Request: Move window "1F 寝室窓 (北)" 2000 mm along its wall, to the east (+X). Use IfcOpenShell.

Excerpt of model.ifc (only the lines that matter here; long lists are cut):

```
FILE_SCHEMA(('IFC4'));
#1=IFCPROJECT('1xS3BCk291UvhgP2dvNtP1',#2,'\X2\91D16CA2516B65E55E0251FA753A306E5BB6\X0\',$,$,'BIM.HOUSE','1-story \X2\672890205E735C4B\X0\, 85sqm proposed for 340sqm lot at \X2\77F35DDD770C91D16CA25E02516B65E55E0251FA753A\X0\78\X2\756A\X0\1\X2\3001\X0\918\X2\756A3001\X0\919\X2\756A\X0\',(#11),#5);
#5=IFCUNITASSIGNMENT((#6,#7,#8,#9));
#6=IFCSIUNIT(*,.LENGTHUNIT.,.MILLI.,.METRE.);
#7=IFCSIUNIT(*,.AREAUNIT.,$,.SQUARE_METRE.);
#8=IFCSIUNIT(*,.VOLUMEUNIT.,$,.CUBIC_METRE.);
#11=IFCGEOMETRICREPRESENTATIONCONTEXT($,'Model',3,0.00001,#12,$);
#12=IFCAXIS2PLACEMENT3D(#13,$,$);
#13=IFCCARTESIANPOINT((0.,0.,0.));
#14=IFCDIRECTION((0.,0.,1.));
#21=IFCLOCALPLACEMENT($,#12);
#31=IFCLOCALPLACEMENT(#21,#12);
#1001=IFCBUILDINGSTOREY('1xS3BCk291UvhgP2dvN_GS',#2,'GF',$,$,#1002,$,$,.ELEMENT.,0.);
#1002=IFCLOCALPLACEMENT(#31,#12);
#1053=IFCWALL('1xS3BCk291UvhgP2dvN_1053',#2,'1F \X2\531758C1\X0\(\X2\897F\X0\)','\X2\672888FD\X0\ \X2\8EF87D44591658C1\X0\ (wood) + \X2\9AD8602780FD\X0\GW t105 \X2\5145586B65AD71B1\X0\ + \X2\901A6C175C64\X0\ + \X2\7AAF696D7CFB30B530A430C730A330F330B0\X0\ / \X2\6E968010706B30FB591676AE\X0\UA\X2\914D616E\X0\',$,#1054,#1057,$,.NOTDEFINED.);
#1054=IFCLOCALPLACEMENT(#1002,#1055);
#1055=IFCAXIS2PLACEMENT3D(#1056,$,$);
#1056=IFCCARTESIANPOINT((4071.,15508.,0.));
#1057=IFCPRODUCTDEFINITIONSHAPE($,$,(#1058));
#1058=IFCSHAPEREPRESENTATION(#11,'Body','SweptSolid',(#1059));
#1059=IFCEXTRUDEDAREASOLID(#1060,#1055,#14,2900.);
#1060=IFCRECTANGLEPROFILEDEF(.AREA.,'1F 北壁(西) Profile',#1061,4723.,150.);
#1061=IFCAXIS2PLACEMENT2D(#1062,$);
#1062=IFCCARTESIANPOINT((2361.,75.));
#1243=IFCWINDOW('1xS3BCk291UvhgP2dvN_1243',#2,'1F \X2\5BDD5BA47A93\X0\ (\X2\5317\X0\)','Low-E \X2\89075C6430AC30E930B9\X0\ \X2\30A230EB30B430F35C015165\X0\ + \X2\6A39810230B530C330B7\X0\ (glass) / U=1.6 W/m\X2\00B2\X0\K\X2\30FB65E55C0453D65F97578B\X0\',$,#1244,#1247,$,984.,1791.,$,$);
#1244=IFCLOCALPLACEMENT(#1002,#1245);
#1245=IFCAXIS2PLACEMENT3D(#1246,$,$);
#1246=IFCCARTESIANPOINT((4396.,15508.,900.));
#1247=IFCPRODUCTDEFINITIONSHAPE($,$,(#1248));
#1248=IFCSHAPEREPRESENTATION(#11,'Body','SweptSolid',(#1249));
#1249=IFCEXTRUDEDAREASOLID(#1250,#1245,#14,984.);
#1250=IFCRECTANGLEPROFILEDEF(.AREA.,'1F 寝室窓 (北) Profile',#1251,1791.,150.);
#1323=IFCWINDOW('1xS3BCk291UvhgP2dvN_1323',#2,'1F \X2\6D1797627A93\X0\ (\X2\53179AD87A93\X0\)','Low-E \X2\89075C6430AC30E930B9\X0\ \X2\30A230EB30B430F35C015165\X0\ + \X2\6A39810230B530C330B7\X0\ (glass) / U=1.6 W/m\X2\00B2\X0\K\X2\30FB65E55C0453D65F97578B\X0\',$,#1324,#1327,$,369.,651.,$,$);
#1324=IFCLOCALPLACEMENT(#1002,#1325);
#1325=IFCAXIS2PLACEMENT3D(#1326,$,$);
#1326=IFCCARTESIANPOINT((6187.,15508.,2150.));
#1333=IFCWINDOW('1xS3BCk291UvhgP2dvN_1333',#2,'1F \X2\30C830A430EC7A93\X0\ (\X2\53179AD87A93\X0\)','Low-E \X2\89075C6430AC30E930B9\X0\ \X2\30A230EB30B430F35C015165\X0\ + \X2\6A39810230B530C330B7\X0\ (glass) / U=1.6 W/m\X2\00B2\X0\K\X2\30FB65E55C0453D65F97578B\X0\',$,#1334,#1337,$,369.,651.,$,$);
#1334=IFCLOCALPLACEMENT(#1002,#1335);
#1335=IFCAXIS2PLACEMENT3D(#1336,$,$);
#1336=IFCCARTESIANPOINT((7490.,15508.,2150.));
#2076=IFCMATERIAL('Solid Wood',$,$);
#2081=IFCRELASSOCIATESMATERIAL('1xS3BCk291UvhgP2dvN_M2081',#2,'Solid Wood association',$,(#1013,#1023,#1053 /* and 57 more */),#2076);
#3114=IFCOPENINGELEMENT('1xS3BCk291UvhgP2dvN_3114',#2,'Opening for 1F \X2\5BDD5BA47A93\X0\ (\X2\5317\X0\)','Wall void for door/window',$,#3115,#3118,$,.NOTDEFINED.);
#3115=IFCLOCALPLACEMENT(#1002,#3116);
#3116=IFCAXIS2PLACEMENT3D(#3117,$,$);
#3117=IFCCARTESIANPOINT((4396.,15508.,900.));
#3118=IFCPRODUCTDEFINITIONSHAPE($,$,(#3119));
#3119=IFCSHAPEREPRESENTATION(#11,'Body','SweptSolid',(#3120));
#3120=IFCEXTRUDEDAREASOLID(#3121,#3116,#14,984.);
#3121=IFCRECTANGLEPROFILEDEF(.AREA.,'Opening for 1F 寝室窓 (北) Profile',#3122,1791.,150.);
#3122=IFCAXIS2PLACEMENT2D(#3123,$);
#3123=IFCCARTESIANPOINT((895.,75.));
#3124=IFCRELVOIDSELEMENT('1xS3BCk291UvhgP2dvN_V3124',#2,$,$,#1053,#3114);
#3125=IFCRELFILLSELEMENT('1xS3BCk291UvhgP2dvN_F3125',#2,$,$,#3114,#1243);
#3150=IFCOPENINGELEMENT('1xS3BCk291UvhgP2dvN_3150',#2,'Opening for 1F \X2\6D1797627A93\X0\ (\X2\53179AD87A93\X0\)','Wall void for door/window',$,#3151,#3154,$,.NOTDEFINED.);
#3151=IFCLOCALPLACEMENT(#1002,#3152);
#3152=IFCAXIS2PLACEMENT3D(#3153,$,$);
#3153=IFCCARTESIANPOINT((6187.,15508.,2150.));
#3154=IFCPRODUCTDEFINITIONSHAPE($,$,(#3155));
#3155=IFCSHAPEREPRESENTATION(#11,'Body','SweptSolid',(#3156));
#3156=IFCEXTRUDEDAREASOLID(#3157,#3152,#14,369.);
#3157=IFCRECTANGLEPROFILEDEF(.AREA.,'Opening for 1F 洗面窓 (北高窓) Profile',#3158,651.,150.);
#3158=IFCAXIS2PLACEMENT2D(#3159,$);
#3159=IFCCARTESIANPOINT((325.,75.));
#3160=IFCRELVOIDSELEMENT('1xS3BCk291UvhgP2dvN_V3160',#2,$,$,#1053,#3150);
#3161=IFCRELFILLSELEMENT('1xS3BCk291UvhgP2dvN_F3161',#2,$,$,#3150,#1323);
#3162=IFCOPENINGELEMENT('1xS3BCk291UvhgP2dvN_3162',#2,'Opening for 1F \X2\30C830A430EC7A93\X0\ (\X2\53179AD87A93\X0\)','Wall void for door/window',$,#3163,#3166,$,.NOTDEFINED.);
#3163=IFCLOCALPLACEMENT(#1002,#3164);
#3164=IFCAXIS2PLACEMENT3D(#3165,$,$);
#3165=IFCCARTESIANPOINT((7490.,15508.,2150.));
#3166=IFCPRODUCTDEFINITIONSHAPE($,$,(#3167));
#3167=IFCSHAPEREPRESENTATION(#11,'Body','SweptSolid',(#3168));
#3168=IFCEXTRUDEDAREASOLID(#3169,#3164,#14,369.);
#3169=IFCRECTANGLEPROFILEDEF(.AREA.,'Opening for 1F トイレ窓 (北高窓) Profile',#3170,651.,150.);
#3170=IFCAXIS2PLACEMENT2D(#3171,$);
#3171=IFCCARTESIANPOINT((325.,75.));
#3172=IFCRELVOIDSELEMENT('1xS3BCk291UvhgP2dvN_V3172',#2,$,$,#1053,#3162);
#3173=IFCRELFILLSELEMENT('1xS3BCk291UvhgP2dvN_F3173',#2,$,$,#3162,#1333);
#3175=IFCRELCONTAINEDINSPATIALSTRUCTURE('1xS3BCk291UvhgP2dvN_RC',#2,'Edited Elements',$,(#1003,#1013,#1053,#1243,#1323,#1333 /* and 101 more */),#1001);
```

```python
import ifcopenshell
import ifcopenshell.api.geometry
import ifcopenshell.util.placement
import ifcopenshell.util.unit

model = ifcopenshell.open("model.ifc")
unit_scale = ifcopenshell.util.unit.calculate_unit_scale(model)

window = model.by_id(1243)
opening = window.FillsVoids[0].RelatingOpeningElement
wall = opening.VoidsElements[0].RelatingBuildingElement

wall_matrix = ifcopenshell.util.placement.get_local_placement(wall.ObjectPlacement)
shift = wall_matrix[:3, 0] * 2 / unit_scale
before = ifcopenshell.util.placement.get_local_placement(window.ObjectPlacement)[:3, 3].copy()

# The window is not placed relative to its opening, so move both.
for product in (opening, window):
    matrix = ifcopenshell.util.placement.get_local_placement(product.ObjectPlacement)
    matrix[:3, 3] += shift
    ifcopenshell.api.geometry.edit_object_placement(model, product=product, matrix=matrix, is_si=False)

after = ifcopenshell.util.placement.get_local_placement(window.ObjectPlacement)[:3, 3]
print("window moved by", (after - before).round(3) + 0.0)

model.write("model_edited.ifc")
```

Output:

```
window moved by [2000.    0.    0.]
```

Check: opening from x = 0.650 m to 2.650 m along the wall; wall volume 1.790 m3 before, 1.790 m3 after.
